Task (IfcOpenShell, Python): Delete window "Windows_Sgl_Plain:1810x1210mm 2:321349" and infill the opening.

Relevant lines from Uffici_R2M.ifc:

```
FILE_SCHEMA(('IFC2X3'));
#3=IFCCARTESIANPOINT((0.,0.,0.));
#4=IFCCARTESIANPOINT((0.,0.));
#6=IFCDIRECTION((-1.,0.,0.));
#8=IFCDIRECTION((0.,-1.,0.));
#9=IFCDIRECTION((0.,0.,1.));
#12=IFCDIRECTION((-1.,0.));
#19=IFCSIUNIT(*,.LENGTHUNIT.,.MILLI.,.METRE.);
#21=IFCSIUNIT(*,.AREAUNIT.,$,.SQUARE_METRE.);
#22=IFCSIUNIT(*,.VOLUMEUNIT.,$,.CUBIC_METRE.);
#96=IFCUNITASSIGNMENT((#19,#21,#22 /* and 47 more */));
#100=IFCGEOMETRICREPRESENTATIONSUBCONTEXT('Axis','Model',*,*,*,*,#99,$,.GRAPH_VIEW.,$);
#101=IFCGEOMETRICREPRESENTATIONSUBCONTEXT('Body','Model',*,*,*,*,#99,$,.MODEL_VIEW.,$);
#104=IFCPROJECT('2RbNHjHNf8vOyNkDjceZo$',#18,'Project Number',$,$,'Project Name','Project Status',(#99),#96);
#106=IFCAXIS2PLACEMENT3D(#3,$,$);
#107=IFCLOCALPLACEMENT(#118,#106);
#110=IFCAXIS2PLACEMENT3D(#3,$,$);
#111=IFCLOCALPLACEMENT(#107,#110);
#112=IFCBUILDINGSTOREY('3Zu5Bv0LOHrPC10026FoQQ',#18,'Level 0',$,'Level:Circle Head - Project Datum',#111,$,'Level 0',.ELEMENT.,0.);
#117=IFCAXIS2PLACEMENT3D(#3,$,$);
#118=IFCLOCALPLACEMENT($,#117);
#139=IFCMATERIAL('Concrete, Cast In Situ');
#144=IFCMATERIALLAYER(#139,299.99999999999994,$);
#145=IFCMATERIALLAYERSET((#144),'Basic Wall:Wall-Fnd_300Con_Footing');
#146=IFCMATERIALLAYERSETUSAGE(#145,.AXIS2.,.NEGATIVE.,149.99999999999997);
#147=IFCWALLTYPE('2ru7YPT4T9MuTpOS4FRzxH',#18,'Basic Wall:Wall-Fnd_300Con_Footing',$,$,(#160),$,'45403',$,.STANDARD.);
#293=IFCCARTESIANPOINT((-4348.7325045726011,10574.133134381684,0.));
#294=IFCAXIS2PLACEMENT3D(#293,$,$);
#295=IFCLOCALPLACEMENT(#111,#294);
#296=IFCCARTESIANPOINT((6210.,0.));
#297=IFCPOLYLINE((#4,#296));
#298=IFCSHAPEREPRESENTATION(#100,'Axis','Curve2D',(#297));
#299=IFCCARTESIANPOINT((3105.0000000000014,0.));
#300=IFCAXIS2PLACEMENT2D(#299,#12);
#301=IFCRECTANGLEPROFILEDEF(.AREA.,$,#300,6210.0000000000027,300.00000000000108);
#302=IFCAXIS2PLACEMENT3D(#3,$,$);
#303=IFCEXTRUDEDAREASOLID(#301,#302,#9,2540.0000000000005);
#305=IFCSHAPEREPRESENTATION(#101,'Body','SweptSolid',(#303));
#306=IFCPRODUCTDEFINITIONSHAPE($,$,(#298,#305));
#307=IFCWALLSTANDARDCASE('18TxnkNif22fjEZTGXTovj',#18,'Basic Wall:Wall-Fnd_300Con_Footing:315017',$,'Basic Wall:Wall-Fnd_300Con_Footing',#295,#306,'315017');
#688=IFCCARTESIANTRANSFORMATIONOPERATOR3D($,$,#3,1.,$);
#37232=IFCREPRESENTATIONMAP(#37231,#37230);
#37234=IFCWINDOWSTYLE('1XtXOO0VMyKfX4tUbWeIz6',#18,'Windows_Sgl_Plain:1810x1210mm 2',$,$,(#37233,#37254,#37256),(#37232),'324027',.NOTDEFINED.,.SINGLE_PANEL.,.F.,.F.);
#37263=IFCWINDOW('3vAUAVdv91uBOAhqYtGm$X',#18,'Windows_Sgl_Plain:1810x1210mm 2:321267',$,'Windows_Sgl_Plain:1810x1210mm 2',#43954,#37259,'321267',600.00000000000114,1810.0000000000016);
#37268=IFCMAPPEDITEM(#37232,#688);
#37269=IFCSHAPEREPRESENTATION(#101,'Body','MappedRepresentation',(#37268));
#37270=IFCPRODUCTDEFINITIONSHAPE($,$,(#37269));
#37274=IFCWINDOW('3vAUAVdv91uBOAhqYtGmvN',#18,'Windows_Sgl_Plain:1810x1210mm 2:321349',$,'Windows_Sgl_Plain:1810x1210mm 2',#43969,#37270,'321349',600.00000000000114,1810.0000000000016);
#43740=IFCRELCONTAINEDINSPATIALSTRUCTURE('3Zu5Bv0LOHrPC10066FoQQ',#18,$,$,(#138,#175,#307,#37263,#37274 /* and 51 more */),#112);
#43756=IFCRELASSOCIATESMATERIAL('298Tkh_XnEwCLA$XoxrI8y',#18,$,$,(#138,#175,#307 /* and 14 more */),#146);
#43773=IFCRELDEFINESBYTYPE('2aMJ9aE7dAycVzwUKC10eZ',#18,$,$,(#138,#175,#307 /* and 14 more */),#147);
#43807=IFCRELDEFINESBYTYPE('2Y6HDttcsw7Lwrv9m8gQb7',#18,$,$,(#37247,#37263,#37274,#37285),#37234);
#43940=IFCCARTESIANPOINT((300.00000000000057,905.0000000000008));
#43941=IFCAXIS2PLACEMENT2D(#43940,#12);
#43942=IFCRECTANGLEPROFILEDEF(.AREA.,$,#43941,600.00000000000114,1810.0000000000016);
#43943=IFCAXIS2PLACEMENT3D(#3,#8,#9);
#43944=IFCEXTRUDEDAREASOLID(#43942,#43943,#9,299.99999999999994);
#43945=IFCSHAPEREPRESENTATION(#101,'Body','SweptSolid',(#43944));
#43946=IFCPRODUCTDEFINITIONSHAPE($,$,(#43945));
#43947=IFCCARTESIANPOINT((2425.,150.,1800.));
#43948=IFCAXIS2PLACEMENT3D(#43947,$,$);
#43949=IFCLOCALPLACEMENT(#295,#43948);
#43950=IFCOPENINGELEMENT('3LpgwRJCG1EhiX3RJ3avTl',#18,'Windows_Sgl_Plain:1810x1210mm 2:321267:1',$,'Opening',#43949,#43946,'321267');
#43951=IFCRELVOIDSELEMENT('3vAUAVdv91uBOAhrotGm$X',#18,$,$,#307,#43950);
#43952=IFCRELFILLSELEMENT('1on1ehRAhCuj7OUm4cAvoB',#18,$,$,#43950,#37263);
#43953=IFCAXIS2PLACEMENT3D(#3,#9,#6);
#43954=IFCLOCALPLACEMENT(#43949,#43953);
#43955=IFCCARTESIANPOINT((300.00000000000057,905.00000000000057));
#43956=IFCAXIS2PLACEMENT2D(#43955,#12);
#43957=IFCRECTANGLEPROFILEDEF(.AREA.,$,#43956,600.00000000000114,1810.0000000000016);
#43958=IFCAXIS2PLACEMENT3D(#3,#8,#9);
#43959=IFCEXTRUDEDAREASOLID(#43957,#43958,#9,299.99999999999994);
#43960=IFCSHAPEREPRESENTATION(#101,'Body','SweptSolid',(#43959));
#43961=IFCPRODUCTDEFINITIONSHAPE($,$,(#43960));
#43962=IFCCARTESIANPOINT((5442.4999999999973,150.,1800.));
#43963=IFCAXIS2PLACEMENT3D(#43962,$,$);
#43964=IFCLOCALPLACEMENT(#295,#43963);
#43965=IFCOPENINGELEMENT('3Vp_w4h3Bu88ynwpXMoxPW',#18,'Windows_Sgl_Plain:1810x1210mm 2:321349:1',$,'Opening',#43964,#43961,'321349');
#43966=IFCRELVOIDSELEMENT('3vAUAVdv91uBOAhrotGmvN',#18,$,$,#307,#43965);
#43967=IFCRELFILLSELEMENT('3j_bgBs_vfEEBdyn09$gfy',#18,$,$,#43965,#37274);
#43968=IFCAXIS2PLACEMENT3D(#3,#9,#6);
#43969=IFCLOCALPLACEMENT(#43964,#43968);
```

```python
import ifcopenshell
import ifcopenshell.api.feature
import ifcopenshell.api.root
import ifcopenshell.geom
import ifcopenshell.util.shape

model = ifcopenshell.open("Uffici_R2M.ifc")
settings = ifcopenshell.geom.settings()


def volume(element):
    """Net volume in cubic metres, openings subtracted."""
    shape = ifcopenshell.geom.create_shape(settings, element)
    return ifcopenshell.util.shape.get_volume(shape.geometry)


window = model.by_guid("3vAUAVdv91uBOAhqYtGmvN")
opening = window.FillsVoids[0].RelatingOpeningElement
wall = opening.VoidsElements[0].RelatingBuildingElement
before = volume(wall)

ifcopenshell.api.root.remove_product(model, product=window)
ifcopenshell.api.feature.remove_feature(model, feature=opening)

after = volume(wall)

print(f"wall volume {before:.3f} -> {after:.3f} m3")

model.write("Uffici_R2M_updated.ifc")
```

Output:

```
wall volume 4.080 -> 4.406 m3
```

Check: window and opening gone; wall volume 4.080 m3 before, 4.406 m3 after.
